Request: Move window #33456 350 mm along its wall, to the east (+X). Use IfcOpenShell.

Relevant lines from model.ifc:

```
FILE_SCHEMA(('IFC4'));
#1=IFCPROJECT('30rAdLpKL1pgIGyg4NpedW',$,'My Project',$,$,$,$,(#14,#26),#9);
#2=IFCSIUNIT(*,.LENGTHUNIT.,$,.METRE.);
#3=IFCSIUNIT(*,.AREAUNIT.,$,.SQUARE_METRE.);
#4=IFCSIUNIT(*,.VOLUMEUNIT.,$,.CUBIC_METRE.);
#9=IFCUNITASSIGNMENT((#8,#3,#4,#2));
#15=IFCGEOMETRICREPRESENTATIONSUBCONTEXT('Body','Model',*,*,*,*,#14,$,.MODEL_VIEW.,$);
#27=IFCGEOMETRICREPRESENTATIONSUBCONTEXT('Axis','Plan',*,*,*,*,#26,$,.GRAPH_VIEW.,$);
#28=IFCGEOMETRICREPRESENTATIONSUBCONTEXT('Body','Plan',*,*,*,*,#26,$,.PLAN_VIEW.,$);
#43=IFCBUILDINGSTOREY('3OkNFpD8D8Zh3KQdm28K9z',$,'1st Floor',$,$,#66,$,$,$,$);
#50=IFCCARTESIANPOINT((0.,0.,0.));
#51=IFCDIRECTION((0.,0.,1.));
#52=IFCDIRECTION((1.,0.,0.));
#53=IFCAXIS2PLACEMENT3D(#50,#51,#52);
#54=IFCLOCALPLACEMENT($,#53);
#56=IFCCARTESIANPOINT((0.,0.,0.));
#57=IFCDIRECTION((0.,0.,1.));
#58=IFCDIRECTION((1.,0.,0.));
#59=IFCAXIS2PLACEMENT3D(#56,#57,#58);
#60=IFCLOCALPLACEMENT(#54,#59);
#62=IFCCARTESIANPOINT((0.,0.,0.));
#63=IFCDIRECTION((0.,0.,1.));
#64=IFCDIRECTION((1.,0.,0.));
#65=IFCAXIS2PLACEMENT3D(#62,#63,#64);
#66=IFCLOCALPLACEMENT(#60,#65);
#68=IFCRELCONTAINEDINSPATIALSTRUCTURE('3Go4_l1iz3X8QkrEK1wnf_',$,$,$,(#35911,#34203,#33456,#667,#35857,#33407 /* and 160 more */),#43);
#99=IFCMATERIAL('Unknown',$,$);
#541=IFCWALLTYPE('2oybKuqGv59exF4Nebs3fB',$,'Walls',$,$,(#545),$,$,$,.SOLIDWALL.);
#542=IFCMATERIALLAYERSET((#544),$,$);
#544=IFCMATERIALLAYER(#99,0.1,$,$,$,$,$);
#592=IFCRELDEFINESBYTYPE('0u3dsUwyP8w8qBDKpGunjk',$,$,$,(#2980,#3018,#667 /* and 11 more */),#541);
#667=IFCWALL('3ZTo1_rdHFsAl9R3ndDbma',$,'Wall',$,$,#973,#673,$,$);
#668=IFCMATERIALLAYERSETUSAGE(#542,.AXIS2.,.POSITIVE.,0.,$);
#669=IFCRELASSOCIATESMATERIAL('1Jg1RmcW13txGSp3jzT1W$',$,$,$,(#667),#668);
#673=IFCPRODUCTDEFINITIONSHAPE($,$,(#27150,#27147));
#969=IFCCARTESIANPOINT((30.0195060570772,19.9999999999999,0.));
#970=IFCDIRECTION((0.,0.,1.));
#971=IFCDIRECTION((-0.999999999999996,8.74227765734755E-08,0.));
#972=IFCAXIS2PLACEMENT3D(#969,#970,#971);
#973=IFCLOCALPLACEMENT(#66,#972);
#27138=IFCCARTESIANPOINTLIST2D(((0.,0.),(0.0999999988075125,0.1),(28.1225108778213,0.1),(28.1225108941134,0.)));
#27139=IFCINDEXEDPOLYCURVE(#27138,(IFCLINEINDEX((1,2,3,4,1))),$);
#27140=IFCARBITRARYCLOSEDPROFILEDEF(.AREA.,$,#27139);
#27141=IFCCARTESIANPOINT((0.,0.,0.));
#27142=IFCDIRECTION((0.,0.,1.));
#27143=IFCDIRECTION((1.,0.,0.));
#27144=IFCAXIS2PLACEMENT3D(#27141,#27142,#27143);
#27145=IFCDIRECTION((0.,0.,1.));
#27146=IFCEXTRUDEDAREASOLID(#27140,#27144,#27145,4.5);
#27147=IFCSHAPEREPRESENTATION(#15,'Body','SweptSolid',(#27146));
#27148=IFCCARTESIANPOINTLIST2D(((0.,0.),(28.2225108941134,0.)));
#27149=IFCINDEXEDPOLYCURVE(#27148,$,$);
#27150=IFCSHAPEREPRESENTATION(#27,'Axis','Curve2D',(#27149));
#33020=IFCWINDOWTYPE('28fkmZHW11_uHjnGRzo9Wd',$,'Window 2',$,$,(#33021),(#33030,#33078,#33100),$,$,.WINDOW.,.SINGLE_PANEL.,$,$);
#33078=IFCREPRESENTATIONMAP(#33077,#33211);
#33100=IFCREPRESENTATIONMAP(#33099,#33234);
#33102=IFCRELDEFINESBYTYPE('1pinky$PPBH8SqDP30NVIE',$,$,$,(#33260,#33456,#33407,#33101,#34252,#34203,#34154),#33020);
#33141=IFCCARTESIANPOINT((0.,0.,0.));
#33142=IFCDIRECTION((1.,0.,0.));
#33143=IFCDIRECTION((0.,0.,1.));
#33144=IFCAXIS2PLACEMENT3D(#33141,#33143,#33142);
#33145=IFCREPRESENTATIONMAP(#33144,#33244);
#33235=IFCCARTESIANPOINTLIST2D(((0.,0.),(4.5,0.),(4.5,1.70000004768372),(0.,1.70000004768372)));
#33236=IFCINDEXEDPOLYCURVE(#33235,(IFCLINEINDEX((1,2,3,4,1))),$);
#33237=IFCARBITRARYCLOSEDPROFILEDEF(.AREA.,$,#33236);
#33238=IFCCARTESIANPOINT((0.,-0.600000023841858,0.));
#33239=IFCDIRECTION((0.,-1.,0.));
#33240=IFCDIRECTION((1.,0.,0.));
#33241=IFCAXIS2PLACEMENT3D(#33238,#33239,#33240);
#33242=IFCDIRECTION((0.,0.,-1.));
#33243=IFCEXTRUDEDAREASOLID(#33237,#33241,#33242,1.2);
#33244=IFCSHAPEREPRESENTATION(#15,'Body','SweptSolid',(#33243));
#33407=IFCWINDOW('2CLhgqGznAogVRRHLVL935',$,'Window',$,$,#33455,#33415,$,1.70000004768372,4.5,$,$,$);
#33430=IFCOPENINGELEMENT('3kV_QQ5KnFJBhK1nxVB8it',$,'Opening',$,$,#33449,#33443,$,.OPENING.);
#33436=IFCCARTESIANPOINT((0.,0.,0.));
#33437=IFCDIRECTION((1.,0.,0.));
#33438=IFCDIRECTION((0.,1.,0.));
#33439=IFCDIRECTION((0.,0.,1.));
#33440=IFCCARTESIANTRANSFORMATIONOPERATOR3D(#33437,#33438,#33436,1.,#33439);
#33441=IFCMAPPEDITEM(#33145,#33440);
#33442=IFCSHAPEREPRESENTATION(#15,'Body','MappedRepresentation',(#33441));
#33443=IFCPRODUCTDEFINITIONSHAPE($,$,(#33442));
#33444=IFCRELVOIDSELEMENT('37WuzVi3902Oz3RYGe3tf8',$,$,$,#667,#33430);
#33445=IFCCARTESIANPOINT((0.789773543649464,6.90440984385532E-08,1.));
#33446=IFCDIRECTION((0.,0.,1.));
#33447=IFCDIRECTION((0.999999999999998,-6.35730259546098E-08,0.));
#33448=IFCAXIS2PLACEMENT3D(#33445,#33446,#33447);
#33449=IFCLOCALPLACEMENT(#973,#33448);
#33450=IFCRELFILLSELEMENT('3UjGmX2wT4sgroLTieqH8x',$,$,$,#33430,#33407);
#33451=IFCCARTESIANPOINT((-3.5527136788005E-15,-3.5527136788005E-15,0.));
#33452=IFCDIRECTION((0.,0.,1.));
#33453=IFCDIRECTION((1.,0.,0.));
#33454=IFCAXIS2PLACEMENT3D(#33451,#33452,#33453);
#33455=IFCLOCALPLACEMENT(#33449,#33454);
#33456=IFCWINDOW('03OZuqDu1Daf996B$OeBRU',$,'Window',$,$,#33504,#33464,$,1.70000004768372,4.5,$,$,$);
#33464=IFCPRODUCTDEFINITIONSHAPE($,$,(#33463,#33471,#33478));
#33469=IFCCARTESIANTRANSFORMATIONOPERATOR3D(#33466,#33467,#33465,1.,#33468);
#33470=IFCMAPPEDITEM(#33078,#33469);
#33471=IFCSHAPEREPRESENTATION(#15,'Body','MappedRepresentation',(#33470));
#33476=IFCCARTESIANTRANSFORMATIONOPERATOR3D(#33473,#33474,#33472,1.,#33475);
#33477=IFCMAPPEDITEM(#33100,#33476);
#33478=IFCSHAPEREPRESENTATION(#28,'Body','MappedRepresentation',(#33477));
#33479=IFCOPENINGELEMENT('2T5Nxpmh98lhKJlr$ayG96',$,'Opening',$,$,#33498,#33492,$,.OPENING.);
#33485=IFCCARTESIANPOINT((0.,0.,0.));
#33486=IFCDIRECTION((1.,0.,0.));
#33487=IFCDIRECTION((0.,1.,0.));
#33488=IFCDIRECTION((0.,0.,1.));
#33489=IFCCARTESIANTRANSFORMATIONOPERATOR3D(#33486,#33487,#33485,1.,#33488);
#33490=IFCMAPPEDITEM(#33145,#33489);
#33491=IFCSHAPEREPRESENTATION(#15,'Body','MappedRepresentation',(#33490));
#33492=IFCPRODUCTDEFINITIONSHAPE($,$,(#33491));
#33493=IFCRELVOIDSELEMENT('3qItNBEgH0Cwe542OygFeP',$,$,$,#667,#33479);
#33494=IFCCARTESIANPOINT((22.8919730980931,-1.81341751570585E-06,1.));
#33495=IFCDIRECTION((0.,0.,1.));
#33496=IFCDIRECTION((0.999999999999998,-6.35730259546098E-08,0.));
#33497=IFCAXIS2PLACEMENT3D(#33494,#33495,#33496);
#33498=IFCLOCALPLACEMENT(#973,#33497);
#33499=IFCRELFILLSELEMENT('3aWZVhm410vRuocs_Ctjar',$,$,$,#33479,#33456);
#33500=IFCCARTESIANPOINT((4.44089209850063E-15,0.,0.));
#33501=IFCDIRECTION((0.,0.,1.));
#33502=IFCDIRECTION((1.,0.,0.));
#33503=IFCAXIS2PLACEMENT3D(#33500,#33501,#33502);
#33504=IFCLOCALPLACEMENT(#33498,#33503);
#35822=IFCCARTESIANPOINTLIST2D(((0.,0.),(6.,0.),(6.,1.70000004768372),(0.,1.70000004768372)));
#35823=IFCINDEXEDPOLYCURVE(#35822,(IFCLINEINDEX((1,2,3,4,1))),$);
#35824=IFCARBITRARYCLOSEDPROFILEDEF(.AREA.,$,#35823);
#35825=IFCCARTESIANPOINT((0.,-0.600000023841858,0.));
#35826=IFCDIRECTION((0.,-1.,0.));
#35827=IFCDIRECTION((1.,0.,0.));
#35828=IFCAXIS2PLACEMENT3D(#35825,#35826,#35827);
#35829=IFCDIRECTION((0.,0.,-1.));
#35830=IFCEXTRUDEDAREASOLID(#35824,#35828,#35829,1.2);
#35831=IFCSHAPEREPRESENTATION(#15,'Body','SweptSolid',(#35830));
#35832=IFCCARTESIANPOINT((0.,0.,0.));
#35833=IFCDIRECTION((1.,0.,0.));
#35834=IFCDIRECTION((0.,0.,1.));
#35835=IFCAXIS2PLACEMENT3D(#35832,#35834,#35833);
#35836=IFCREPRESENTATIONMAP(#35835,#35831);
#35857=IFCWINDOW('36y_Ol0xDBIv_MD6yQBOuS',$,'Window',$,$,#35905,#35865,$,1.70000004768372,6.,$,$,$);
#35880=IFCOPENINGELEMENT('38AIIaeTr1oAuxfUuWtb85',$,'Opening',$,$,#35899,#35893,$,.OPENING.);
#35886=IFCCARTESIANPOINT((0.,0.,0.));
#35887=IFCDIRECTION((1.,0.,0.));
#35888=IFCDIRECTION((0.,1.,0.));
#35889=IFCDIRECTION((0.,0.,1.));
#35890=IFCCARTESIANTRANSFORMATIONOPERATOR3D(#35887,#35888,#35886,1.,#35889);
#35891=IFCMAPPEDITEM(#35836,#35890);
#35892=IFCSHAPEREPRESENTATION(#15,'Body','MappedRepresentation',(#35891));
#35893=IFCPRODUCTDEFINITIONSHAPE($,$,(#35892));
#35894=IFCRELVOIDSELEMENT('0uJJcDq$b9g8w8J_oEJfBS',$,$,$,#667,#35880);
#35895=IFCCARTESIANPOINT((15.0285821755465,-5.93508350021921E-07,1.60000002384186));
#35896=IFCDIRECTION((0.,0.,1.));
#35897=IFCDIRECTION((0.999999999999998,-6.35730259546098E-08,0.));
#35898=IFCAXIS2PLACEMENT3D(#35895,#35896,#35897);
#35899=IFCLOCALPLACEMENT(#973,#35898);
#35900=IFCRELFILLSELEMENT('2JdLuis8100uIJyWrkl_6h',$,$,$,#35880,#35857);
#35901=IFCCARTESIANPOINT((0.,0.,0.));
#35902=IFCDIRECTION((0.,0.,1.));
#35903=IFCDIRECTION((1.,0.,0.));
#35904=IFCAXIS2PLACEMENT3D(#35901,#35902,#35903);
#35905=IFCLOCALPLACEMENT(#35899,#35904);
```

```python
import ifcopenshell
import ifcopenshell.api.geometry
import ifcopenshell.util.placement

model = ifcopenshell.open("model.ifc")

window = model.by_guid("03OZuqDu1Daf996B$OeBRU")
opening = window.FillsVoids[0].RelatingOpeningElement
wall = opening.VoidsElements[0].RelatingBuildingElement

wall_matrix = ifcopenshell.util.placement.get_local_placement(wall.ObjectPlacement)
shift = wall_matrix[:3, 0] * -0.35
before = ifcopenshell.util.placement.get_local_placement(window.ObjectPlacement)[:3, 3].copy()

# The window is placed relative to its opening, so it follows when the opening moves.
matrix = ifcopenshell.util.placement.get_local_placement(opening.ObjectPlacement)
matrix[:3, 3] += shift
ifcopenshell.api.geometry.edit_object_placement(
    model, product=opening, matrix=matrix, is_si=False, should_transform_children=True
)

after = ifcopenshell.util.placement.get_local_placement(window.ObjectPlacement)[:3, 3]
print("window moved by", (after - before).round(3) + 0.0)

model.write("model_edited.ifc")
```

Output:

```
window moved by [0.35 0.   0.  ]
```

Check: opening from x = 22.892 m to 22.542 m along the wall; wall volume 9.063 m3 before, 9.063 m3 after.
